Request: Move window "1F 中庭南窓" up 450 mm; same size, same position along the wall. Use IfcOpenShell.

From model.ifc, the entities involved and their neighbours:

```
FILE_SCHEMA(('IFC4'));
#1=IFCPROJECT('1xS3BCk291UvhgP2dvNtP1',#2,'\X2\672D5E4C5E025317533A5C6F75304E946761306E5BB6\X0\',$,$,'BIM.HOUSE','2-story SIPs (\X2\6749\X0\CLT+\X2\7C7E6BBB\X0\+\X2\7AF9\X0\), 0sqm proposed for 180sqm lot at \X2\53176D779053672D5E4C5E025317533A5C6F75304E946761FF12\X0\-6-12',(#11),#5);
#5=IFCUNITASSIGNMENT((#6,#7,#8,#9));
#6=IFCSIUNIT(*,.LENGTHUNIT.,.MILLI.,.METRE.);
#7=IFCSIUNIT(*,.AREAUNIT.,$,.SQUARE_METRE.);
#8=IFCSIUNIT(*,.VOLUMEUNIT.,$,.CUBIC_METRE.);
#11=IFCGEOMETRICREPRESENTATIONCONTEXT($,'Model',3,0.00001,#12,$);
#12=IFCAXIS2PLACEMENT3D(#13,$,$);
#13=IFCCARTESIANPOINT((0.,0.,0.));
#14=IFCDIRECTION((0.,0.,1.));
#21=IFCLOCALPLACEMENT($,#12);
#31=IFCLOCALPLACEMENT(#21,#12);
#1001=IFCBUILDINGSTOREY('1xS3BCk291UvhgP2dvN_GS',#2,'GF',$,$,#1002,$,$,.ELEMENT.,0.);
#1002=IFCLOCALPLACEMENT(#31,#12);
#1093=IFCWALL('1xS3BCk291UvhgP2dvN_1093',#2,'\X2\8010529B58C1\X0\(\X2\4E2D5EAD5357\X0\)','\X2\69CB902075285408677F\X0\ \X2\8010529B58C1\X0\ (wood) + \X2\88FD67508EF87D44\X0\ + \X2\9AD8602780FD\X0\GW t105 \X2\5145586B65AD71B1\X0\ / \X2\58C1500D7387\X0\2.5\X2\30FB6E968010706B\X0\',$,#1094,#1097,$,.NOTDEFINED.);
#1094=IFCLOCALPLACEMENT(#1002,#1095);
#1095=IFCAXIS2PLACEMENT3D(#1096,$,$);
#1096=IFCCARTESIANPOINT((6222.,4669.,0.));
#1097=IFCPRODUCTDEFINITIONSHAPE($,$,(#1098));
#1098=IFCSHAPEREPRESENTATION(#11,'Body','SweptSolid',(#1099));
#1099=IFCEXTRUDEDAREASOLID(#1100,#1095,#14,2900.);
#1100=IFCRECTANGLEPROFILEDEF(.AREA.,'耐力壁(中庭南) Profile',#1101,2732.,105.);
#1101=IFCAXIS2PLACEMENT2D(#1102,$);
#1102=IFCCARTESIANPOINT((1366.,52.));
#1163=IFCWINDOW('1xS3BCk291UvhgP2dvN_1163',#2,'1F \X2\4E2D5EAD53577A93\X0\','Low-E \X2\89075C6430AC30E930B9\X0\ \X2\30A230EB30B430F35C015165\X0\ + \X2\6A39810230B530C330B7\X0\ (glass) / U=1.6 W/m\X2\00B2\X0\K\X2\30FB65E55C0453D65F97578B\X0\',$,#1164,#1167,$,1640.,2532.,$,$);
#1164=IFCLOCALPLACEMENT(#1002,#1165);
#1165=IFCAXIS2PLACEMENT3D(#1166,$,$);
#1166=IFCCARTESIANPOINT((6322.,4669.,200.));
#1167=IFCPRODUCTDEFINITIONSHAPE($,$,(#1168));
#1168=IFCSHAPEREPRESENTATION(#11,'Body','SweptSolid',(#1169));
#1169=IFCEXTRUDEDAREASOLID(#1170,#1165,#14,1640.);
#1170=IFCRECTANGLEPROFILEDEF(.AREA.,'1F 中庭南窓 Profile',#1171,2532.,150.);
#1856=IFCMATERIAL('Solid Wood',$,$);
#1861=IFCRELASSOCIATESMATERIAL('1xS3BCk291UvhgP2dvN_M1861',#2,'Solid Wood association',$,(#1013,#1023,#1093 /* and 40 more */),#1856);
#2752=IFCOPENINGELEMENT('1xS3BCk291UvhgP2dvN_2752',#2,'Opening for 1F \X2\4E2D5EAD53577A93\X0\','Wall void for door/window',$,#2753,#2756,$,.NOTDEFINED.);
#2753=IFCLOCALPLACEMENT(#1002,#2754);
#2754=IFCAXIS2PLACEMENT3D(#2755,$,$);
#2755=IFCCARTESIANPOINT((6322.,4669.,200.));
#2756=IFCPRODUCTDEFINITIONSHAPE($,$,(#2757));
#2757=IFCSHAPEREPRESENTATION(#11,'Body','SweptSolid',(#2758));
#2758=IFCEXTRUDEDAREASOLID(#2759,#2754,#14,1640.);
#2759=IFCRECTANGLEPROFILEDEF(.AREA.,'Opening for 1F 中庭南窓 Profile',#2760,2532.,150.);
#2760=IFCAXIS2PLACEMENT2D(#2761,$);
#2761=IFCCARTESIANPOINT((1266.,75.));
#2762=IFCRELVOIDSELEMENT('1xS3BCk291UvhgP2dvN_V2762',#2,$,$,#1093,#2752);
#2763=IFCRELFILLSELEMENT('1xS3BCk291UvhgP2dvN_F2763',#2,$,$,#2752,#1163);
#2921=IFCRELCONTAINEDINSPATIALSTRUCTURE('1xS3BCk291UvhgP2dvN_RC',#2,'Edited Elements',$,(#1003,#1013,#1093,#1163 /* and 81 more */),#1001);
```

```python
import numpy as np
import ifcopenshell
import ifcopenshell.api.geometry
import ifcopenshell.util.placement
import ifcopenshell.util.unit

model = ifcopenshell.open("model.ifc")
unit_scale = ifcopenshell.util.unit.calculate_unit_scale(model)

window = model.by_guid("1xS3BCk291UvhgP2dvN_1163")
opening = window.FillsVoids[0].RelatingOpeningElement
dz = 450.0

shift = np.array([0.0, 0.0, dz])
# The window is not placed relative to its opening, so move both.
for product in (opening, window):
    matrix = ifcopenshell.util.placement.get_local_placement(product.ObjectPlacement)
    matrix[:3, 3] += shift
    ifcopenshell.api.geometry.edit_object_placement(model, product=product, matrix=matrix, is_si=False)

print(f"moved by {dz * unit_scale:+.3f} m")

model.write("model-out.ifc")
```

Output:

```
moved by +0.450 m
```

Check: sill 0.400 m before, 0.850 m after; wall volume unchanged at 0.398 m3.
